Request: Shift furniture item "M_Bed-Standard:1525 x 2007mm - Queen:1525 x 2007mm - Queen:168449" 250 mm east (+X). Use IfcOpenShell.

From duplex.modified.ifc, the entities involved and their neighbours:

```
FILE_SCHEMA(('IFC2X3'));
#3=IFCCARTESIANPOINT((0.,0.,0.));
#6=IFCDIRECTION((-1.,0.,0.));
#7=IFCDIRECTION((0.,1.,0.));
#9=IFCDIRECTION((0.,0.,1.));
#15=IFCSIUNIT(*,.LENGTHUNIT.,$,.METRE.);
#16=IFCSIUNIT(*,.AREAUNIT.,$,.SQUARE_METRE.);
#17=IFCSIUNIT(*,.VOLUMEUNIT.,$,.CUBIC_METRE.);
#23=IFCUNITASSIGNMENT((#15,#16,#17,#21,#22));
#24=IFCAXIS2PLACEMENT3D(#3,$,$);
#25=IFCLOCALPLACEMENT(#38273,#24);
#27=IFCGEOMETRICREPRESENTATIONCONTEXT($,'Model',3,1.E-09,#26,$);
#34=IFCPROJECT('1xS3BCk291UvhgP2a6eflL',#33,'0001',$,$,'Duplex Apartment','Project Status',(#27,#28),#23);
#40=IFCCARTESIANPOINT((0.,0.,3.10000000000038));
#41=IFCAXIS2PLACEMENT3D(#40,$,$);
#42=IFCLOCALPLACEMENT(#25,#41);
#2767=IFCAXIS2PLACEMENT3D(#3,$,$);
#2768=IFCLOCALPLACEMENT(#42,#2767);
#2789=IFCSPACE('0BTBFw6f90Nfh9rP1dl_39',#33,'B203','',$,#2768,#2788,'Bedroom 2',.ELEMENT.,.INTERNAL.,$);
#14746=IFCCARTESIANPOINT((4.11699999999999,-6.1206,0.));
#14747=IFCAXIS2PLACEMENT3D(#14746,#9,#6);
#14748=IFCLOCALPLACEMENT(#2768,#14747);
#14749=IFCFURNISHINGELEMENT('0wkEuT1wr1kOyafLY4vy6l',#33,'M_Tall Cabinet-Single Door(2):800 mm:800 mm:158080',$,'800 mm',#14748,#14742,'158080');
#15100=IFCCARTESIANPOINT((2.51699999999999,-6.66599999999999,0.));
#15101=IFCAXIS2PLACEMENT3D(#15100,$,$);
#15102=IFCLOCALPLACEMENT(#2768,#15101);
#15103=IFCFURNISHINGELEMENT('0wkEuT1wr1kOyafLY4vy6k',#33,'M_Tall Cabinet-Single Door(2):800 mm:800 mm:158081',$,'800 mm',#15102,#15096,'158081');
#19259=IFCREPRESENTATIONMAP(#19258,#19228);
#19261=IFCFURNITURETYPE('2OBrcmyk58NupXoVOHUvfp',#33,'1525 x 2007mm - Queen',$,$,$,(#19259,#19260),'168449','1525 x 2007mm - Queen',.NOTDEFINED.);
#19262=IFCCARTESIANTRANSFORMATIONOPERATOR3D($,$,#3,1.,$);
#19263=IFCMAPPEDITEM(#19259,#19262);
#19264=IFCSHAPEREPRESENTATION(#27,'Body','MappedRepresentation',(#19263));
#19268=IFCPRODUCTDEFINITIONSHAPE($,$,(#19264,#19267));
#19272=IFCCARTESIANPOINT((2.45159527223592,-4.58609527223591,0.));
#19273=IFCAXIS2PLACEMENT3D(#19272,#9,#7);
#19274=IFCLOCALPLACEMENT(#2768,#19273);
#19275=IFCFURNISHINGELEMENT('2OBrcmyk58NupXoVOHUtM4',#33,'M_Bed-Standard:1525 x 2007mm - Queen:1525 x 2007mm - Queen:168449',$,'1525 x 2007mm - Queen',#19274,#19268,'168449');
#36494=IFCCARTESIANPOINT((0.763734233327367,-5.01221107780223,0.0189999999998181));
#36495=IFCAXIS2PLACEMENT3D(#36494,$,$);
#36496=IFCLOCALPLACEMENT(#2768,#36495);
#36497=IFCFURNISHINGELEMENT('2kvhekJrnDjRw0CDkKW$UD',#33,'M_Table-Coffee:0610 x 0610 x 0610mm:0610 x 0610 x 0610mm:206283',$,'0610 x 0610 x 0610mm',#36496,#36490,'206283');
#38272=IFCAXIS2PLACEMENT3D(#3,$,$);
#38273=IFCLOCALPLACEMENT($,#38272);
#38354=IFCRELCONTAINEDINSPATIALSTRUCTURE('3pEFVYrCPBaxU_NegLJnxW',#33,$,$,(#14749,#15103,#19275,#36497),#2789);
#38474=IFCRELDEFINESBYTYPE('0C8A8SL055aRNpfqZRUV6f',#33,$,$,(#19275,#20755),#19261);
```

```python
import ifcopenshell
import ifcopenshell.api.geometry
import ifcopenshell.util.placement
import ifcopenshell.util.unit

model = ifcopenshell.open("duplex.modified.ifc")
unit_scale = ifcopenshell.util.unit.calculate_unit_scale(model)

item = model.by_guid("2OBrcmyk58NupXoVOHUtM4")
matrix = ifcopenshell.util.placement.get_local_placement(item.ObjectPlacement)
matrix[0, 3] += 0.25 / unit_scale
ifcopenshell.api.geometry.edit_object_placement(model, product=item, matrix=matrix, is_si=False)

print(ifcopenshell.util.placement.get_local_placement(item.ObjectPlacement).round(3) + 0.0)

model.write("duplex.modified_rev.ifc")
```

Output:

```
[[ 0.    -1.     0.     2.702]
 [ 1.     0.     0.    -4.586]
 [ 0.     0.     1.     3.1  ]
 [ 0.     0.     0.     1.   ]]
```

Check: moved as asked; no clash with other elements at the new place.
